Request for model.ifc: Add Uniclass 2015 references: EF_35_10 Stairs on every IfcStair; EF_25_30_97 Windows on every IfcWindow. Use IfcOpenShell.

First a look at what the model holds.

```python
import ifcopenshell

model = ifcopenshell.open("model.ifc")
print(model.schema)
print("classifications:", [c.Name for c in model.by_type("IfcClassification")])
for ifc_class in ("IfcDoor", "IfcRoof", "IfcStair", "IfcWall", "IfcWindow"):
    print(ifc_class, len(model.by_type(ifc_class)))
```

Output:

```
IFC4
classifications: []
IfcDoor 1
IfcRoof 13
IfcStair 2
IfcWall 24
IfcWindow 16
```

```python
import ifcopenshell
import ifcopenshell.api.classification

model = ifcopenshell.open("model.ifc")

system = ifcopenshell.api.classification.add_classification(model, classification="Uniclass 2015")

codes = {
    "IfcStair": ("EF_35_10", "Stairs"),
    "IfcWindow": ("EF_25_30_97", "Windows"),
}
for ifc_class, (code, name) in codes.items():
    products = model.by_type(ifc_class)
    ifcopenshell.api.classification.add_reference(
        model, products=products, classification=system, identification=code, name=name
    )
    print(code, len(products))

model.write("model_updated.ifc")
```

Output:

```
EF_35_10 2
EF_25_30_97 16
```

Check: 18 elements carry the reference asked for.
